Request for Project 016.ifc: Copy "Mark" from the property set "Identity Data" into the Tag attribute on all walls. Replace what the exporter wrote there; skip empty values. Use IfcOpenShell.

First a look at what the model holds.

```python
import ifcopenshell
import ifcopenshell.util.element

model = ifcopenshell.open("Project 016.ifc")
print(model.schema)
walls = model.by_type("IfcWall")
print(len(walls), "walls")
for e in walls[:8]:
    source = ifcopenshell.util.element.get_pset(e, "Identity Data", "Mark")
    target = e.Tag
    print(e.id(), repr(source), repr(target), sep=" | ")
```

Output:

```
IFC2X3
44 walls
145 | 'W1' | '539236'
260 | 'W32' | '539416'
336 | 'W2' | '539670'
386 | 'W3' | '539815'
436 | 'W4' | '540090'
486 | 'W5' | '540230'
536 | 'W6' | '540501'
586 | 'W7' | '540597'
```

```python
import ifcopenshell
import ifcopenshell.util.element

model = ifcopenshell.open("Project 016.ifc")

count = 0
for e in model.by_type("IfcWall"):
    value = ifcopenshell.util.element.get_pset(e, "Identity Data", "Mark")
    current = e.Tag
    if not value or not value.strip() or current == value:
        continue
    e.Tag = value
    count += 1

print(count, "walls updated")

model.write("Project 016_v2.ifc")
```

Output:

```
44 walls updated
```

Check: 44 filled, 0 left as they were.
